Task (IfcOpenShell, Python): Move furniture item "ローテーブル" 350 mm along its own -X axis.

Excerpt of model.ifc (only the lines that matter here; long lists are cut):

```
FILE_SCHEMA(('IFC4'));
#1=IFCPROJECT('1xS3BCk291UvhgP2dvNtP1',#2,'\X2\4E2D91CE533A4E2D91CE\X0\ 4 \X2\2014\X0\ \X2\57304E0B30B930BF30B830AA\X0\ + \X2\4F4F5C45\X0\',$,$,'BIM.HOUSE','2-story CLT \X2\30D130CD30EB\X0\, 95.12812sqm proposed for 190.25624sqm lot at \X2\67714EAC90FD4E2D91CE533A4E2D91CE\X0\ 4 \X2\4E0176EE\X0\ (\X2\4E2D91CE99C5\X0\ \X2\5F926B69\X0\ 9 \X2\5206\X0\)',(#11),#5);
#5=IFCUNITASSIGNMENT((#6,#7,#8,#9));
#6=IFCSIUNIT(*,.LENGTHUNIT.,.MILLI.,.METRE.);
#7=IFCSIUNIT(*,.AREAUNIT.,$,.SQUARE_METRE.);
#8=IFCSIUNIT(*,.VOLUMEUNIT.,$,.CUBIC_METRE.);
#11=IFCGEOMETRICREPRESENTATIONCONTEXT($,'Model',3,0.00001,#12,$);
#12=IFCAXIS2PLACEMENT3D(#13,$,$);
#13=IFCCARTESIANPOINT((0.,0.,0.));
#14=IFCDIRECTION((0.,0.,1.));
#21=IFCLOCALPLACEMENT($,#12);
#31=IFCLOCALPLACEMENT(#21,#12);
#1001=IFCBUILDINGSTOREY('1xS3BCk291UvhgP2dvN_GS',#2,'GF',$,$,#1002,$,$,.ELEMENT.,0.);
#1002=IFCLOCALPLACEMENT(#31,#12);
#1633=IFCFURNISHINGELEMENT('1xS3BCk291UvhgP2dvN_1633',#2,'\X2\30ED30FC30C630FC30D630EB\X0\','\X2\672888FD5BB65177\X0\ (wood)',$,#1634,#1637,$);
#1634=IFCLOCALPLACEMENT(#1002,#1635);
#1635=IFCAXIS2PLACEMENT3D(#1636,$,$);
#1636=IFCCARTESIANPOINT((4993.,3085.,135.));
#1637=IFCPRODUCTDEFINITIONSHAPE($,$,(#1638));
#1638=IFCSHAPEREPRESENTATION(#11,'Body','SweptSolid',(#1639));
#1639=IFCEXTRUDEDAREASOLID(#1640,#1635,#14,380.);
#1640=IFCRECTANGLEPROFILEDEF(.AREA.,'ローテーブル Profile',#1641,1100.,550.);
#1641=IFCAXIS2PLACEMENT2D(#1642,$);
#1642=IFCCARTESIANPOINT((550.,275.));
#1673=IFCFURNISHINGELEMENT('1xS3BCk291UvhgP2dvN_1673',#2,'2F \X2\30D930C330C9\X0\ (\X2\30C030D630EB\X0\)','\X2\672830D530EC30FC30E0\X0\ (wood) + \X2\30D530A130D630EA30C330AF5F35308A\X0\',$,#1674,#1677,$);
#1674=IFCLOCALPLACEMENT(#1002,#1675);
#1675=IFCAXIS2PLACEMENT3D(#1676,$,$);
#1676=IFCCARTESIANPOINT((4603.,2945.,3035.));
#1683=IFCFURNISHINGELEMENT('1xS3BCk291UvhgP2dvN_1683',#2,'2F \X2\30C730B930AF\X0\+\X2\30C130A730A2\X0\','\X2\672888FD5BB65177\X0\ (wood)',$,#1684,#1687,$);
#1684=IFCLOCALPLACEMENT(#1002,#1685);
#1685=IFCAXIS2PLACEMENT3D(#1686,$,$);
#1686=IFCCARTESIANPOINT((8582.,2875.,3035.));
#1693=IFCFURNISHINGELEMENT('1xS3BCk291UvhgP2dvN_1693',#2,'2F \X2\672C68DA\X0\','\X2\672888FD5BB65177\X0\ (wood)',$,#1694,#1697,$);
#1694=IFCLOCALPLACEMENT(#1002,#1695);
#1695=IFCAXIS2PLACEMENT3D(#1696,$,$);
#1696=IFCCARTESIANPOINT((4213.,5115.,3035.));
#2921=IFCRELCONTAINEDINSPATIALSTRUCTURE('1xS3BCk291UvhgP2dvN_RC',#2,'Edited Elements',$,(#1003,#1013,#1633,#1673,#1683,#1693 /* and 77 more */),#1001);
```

```python
import ifcopenshell
import ifcopenshell.api.geometry
import ifcopenshell.util.placement

model = ifcopenshell.open("model.ifc")

item = model.by_guid("1xS3BCk291UvhgP2dvN_1633")
matrix = ifcopenshell.util.placement.get_local_placement(item.ObjectPlacement)
matrix[:3, 3] -= matrix[:3, 0] * 350.0
ifcopenshell.api.geometry.edit_object_placement(model, product=item, matrix=matrix, is_si=False)

print(ifcopenshell.util.placement.get_local_placement(item.ObjectPlacement).round(3) + 0.0)

model.write("model_updated.ifc")
```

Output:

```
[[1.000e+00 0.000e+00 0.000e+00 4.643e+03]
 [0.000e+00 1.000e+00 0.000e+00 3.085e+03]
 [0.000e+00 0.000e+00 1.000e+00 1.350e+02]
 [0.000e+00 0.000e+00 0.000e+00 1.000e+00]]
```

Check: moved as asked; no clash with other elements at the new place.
